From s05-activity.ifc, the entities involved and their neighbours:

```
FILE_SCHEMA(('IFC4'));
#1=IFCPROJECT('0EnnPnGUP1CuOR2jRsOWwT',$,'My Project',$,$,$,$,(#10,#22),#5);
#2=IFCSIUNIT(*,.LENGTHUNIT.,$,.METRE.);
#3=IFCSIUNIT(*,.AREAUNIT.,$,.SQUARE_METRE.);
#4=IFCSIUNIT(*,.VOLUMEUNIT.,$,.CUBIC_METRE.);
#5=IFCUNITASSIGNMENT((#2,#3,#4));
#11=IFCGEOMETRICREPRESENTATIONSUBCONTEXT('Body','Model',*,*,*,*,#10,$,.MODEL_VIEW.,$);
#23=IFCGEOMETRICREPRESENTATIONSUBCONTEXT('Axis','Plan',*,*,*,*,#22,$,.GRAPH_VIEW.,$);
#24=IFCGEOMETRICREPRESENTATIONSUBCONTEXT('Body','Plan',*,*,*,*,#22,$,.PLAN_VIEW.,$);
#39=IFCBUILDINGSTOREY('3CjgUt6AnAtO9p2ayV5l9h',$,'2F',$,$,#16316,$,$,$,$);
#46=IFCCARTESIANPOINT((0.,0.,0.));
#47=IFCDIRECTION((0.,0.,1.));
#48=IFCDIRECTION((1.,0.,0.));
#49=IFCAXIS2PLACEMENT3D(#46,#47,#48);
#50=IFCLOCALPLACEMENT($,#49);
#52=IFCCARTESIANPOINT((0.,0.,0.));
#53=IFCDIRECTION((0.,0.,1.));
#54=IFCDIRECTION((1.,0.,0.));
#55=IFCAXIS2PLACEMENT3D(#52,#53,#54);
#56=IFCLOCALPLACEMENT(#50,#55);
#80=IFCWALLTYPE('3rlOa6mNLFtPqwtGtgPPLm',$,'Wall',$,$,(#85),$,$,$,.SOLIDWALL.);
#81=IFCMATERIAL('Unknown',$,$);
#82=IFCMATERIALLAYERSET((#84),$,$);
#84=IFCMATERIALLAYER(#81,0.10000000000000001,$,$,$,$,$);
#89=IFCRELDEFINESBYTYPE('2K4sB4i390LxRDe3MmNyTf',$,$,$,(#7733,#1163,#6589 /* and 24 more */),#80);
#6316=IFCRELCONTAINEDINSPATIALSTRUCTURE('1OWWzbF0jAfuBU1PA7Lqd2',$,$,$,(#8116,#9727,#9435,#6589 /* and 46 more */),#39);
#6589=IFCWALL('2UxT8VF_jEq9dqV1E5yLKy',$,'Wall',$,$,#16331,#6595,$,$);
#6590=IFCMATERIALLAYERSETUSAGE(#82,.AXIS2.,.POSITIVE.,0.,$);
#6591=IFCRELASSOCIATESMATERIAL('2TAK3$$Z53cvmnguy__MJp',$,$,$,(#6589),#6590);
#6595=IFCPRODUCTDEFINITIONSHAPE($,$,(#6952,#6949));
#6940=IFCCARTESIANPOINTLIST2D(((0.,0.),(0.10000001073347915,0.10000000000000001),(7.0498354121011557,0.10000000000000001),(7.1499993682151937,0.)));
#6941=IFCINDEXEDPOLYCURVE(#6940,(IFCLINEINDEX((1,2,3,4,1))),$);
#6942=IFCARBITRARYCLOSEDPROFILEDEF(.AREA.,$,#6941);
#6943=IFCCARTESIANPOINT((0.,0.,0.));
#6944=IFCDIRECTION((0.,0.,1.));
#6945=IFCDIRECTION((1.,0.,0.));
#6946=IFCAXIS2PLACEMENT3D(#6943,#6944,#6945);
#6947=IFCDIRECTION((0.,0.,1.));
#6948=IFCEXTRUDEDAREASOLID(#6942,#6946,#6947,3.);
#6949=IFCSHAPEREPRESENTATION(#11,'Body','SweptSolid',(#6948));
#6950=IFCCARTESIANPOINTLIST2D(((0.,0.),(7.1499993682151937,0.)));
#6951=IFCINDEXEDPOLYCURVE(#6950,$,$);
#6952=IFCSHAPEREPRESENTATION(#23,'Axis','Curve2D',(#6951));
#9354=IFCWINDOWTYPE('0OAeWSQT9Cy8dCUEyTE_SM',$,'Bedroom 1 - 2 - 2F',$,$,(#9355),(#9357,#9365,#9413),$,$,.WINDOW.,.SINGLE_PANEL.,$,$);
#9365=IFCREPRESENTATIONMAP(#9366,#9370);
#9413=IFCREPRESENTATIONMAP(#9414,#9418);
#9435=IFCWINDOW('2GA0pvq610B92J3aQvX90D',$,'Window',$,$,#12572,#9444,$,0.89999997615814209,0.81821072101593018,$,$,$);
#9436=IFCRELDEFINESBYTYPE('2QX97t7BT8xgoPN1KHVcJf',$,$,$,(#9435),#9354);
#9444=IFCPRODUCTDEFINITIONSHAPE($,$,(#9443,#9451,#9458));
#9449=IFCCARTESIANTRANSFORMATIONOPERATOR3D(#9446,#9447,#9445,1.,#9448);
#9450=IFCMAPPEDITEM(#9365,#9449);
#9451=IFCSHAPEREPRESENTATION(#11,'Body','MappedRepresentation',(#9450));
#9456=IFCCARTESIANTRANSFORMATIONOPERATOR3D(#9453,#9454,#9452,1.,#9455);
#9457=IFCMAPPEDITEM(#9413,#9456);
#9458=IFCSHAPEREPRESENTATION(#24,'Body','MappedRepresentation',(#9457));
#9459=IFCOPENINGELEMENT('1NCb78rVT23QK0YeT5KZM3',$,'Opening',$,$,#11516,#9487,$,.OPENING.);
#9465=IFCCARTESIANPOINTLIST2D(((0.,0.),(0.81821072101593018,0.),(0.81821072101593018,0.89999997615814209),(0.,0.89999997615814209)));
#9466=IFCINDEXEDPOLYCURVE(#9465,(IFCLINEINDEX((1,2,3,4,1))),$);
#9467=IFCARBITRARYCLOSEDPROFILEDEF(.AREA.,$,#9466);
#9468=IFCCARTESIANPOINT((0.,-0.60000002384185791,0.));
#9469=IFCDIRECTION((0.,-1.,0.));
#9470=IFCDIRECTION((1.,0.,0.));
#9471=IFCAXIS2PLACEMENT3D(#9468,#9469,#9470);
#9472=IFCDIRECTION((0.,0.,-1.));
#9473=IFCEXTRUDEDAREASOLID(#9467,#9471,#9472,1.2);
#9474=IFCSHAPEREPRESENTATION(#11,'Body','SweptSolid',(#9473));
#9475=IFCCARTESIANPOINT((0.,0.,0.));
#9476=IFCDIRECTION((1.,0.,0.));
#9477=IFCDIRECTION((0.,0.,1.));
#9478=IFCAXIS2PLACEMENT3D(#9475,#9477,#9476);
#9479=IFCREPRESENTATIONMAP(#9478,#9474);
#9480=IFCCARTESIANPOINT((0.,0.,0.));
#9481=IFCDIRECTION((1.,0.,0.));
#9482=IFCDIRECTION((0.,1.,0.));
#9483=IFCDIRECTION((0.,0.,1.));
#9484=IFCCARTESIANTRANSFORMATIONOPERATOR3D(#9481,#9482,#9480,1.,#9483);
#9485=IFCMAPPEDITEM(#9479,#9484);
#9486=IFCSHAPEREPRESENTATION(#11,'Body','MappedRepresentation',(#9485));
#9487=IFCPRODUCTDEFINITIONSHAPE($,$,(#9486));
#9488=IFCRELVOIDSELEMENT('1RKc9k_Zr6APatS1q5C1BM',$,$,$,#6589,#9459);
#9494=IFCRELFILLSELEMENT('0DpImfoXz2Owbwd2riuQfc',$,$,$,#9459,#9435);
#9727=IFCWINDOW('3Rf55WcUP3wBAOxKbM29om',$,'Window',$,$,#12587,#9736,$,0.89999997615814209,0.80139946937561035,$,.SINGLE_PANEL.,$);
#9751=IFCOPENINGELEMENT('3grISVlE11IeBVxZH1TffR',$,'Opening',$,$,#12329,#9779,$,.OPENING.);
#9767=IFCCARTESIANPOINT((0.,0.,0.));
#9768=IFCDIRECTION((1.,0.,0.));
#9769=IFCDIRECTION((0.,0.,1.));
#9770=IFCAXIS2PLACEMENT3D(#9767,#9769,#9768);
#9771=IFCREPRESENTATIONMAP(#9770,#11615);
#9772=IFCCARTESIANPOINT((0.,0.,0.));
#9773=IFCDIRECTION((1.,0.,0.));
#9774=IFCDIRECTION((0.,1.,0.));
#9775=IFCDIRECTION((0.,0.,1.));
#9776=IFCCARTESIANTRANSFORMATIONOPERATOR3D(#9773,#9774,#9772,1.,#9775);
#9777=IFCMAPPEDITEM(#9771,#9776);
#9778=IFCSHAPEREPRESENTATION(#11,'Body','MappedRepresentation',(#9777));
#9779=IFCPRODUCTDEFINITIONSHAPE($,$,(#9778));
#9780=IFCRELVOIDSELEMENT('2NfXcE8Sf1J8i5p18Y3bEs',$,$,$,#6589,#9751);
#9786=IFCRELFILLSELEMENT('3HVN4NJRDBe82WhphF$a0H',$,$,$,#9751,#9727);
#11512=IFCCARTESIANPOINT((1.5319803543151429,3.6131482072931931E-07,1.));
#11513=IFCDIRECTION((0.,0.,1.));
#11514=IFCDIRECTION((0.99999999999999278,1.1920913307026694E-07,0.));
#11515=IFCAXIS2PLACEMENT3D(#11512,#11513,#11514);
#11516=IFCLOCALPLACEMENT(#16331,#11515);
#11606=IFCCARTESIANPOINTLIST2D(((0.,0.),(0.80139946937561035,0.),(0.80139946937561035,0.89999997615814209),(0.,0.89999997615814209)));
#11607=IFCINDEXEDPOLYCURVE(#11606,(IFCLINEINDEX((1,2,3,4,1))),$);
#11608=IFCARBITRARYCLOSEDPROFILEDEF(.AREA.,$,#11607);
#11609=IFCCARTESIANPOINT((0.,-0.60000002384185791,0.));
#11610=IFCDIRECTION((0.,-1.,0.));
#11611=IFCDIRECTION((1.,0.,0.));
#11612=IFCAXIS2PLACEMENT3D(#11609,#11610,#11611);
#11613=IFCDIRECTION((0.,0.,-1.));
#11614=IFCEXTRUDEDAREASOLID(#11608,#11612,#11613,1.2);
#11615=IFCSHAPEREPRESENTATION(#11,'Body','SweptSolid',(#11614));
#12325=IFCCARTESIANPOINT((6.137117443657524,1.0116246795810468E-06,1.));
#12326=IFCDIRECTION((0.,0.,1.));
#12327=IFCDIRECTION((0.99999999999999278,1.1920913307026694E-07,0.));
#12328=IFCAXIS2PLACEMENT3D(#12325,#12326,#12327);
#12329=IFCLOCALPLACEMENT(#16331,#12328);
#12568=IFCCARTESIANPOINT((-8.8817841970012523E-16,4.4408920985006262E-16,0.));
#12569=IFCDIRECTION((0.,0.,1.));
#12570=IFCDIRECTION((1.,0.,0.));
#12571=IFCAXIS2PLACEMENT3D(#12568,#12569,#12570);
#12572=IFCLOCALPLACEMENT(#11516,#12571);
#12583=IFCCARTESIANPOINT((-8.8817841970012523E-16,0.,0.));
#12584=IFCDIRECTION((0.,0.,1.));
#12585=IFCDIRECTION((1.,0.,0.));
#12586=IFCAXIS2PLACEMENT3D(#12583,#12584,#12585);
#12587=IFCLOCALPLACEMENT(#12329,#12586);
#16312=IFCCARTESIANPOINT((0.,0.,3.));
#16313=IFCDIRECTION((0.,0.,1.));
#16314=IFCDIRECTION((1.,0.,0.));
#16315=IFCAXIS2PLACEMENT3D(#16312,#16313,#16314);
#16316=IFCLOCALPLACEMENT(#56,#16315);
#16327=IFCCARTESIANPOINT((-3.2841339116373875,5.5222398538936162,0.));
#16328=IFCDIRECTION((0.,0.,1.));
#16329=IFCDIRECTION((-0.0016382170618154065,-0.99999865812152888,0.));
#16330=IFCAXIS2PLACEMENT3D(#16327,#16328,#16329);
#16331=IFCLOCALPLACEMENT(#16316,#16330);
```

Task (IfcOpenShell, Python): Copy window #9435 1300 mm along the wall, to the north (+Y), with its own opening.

```python
import ifcopenshell
import ifcopenshell.api.feature
import ifcopenshell.api.geometry
import ifcopenshell.api.root
import ifcopenshell.geom
import ifcopenshell.util.element
import ifcopenshell.util.placement
import ifcopenshell.util.shape
import ifcopenshell.util.unit

model = ifcopenshell.open("s05-activity.ifc")
unit_scale = ifcopenshell.util.unit.calculate_unit_scale(model)
settings = ifcopenshell.geom.settings()


def volume(element):
    """Net volume in cubic metres, openings subtracted."""
    shape = ifcopenshell.geom.create_shape(settings, element)
    return ifcopenshell.util.shape.get_volume(shape.geometry)


window = model.by_guid("2GA0pvq610B92J3aQvX90D")
opening = window.FillsVoids[0].RelatingOpeningElement
wall = opening.VoidsElements[0].RelatingBuildingElement
before = volume(wall)
shift = ifcopenshell.util.placement.get_local_placement(wall.ObjectPlacement)[:3, 0] * -1.3 / unit_scale

# copy_class copies the void relationship, type, container and properties, but no geometry.
new_opening = ifcopenshell.api.root.copy_class(model, product=opening)
new_opening.Representation = ifcopenshell.util.element.copy_deep(
    model, opening.Representation, exclude=["IfcGeometricRepresentationContext", "IfcRepresentationMap"]
)
new_window = ifcopenshell.api.root.copy_class(model, product=window)
new_window.Representation = ifcopenshell.util.element.copy_deep(
    model, window.Representation, exclude=["IfcGeometricRepresentationContext", "IfcRepresentationMap"]
)
ifcopenshell.api.feature.add_filling(model, opening=new_opening, element=new_window)

for old, new in ((opening, new_opening), (window, new_window)):
    matrix = ifcopenshell.util.placement.get_local_placement(old.ObjectPlacement)
    matrix[:3, 3] += shift
    ifcopenshell.api.geometry.edit_object_placement(model, product=new, matrix=matrix, is_si=False)

after = volume(wall)

print(f"wall volume {before:.3f} -> {after:.3f} m3")

model.write("s05-activity_edited.ifc")
```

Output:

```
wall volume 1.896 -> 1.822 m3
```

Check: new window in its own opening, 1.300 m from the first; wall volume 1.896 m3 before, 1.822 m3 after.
